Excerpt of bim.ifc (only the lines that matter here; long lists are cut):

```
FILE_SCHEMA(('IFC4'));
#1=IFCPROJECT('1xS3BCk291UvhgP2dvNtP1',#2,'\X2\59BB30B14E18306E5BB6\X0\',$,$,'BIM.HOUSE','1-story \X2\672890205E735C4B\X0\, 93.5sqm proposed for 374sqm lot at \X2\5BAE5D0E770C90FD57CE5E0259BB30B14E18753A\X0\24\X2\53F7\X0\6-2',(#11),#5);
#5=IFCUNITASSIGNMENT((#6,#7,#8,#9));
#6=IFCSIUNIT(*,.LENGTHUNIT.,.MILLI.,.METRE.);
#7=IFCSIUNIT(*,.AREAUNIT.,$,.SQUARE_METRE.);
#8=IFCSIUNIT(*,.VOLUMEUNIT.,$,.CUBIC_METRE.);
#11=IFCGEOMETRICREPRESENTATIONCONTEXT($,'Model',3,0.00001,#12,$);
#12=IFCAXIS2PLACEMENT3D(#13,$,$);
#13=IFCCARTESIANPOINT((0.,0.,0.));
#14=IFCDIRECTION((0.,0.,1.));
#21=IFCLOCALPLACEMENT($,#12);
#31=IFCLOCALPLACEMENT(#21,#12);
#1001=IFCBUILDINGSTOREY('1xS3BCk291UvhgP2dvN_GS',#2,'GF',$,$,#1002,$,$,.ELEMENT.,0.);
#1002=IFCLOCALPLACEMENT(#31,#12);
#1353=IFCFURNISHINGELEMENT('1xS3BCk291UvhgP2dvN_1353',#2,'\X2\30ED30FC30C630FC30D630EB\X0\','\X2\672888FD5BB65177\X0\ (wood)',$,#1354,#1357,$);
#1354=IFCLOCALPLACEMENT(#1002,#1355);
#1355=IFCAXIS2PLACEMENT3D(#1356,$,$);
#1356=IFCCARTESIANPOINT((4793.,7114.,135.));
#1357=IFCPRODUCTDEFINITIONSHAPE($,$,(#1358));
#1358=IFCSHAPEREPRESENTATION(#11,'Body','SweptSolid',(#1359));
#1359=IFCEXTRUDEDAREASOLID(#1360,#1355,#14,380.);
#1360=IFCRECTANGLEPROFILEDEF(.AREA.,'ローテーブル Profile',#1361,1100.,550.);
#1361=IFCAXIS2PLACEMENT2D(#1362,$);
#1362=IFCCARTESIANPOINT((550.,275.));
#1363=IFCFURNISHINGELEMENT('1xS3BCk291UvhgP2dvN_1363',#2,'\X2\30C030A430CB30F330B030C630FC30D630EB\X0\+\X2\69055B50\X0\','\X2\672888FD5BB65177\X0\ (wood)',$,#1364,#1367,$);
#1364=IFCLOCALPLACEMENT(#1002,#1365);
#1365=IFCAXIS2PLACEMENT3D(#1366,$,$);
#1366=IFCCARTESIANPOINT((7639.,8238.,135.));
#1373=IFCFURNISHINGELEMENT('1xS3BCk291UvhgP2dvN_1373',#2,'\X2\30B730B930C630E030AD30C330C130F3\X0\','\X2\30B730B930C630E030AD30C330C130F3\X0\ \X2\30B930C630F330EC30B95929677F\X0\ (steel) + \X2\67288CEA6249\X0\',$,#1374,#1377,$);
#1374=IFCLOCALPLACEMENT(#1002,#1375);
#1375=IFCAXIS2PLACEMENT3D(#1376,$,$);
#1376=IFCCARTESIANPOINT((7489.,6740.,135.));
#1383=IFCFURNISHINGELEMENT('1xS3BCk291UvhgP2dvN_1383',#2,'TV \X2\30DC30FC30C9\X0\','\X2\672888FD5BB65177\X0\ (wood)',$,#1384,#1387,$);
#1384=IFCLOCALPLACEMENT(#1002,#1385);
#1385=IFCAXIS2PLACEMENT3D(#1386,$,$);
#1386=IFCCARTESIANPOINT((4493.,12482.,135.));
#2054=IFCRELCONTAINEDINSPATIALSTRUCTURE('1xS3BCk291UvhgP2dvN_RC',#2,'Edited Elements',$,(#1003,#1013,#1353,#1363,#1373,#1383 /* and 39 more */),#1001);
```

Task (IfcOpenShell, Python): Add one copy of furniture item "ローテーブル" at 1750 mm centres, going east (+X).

```python
import numpy as np
import ifcopenshell
import ifcopenshell.api.geometry
import ifcopenshell.api.root
import ifcopenshell.util.element
import ifcopenshell.util.placement

model = ifcopenshell.open("bim.ifc")


def reuse_history(source, copy):
    """copy_class also copies each property set's owner history, people and application; keep the originals."""
    for rel in copy.IsDefinedBy:
        if rel.is_a("IfcRelDefinesByProperties") and (history := rel.RelatingPropertyDefinition.OwnerHistory):
            rel.RelatingPropertyDefinition.OwnerHistory = source.OwnerHistory
            ifcopenshell.util.element.remove_deep2(model, history)


source = model.by_guid("1xS3BCk291UvhgP2dvN_1353")
base = ifcopenshell.util.placement.get_local_placement(source.ObjectPlacement)
step = np.array([1.0, 0.0, 0.0]) * 1750.0

for i in range(1, 2):
    copy = ifcopenshell.api.root.copy_class(model, product=source)
    copy.Representation = ifcopenshell.util.element.copy_deep(
        model, source.Representation, exclude=["IfcGeometricRepresentationContext", "IfcRepresentationMap"]
    )
    reuse_history(source, copy)
    matrix = base.copy()
    matrix[:3, 3] += i * step
    print("added at", matrix[:3, 3].round(3) + 0.0)
    ifcopenshell.api.geometry.edit_object_placement(model, product=copy, matrix=matrix, is_si=False)

model.write("bim_edited.ifc")
```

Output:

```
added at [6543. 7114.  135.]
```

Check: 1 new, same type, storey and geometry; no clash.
